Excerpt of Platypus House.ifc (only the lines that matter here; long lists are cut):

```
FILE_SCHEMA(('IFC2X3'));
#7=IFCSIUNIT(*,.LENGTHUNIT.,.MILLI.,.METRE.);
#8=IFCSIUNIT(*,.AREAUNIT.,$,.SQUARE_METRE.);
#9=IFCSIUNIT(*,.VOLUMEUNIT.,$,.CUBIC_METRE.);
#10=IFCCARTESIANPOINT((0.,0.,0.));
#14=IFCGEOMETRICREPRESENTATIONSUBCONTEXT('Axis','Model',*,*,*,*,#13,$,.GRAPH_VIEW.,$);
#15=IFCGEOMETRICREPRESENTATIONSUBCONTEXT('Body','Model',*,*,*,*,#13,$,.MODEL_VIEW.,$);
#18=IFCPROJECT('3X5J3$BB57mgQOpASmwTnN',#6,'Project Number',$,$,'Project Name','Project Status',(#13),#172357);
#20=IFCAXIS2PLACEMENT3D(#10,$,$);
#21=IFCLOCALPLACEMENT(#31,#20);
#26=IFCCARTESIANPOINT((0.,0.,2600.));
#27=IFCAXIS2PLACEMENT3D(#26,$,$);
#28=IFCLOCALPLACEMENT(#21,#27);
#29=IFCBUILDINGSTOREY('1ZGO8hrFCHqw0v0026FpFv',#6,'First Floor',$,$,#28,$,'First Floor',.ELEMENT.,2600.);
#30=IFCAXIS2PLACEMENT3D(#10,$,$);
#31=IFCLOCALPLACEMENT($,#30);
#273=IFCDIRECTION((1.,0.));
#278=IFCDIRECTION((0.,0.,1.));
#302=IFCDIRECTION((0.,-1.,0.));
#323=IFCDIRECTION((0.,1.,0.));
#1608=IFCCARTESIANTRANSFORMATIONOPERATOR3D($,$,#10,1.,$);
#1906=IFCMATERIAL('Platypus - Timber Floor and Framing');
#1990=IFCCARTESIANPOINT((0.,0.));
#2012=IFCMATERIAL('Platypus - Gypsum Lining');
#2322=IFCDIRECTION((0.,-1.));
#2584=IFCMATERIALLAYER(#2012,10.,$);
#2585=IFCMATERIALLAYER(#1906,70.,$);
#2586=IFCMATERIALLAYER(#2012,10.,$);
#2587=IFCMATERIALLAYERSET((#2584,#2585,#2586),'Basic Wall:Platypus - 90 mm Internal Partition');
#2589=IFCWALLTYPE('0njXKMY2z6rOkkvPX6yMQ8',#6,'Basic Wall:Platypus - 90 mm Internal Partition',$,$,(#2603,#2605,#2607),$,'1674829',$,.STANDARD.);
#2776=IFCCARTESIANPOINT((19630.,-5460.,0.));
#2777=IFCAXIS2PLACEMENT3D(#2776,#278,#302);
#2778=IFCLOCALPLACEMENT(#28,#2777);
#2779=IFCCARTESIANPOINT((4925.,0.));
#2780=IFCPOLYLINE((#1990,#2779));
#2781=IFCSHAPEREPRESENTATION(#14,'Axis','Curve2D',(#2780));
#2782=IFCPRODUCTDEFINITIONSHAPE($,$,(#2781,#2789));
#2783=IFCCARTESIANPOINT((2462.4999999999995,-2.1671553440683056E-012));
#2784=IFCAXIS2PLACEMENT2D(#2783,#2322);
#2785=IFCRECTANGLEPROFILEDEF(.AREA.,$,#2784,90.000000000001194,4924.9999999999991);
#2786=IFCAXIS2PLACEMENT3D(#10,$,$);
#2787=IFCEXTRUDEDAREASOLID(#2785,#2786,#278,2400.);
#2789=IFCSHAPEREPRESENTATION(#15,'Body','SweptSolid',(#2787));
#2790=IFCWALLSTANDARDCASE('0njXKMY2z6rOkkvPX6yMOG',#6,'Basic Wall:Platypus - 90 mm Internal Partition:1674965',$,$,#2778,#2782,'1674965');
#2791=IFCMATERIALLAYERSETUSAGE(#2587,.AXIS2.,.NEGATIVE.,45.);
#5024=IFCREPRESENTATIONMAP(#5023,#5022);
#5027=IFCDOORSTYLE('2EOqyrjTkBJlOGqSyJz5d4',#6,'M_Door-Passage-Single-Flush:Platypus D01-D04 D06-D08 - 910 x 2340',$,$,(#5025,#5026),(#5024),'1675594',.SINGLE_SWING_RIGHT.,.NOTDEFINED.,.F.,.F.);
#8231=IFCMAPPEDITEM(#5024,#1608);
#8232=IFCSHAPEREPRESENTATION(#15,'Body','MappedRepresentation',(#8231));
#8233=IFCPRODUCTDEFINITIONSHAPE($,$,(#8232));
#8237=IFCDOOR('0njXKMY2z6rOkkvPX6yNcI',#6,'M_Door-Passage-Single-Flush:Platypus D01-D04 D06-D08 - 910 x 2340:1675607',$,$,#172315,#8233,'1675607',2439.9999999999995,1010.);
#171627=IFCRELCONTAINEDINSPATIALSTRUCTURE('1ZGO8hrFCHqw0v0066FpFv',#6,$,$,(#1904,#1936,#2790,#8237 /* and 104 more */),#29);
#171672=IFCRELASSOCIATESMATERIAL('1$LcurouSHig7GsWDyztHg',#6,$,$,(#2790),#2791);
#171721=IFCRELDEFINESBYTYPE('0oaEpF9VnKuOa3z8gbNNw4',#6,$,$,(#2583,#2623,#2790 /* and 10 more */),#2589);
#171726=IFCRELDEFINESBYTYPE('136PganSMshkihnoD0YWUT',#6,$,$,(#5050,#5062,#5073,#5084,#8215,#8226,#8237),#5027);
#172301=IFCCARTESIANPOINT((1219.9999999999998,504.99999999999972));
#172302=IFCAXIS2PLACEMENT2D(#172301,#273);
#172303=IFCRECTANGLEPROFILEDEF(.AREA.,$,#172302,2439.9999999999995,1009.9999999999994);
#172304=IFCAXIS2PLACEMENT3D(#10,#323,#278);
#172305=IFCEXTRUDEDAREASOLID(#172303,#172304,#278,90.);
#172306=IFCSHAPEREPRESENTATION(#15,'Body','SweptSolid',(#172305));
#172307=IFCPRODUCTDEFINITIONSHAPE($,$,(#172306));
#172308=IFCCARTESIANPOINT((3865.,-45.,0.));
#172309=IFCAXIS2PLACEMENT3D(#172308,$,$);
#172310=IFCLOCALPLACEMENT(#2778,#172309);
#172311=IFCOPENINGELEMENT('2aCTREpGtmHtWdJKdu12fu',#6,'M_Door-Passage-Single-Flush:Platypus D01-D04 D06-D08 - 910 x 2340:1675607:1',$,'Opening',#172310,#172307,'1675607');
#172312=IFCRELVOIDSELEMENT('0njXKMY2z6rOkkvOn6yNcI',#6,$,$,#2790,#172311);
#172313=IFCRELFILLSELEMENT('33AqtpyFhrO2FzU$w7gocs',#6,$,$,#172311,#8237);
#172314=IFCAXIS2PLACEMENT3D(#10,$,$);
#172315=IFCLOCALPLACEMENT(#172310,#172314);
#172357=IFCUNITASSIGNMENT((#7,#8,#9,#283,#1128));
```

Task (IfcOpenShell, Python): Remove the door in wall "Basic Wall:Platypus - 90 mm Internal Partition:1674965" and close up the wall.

```python
import ifcopenshell
import ifcopenshell.api.feature
import ifcopenshell.api.root
import ifcopenshell.geom
import ifcopenshell.util.shape

model = ifcopenshell.open("Platypus House.ifc")
settings = ifcopenshell.geom.settings()


def volume(element):
    """Net volume in cubic metres, openings subtracted."""
    shape = ifcopenshell.geom.create_shape(settings, element)
    return ifcopenshell.util.shape.get_volume(shape.geometry)


door = model.by_guid("0njXKMY2z6rOkkvPX6yNcI")
opening = door.FillsVoids[0].RelatingOpeningElement
wall = opening.VoidsElements[0].RelatingBuildingElement
before = volume(wall)

ifcopenshell.api.root.remove_product(model, product=door)
ifcopenshell.api.feature.remove_feature(model, feature=opening)

after = volume(wall)

print(f"wall volume {before:.3f} -> {after:.3f} m3")

model.write("Platypus House_v2.ifc")
```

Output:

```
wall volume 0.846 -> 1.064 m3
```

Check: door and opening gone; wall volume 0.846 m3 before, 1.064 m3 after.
